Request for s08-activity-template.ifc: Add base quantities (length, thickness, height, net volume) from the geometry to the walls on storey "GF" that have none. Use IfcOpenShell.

First a look at what the model holds.

```python
import ifcopenshell
import ifcopenshell.util.element
import ifcopenshell.util.unit

model = ifcopenshell.open("s08-activity-template.ifc")
print(model.schema)
for unit_type in ("LENGTHUNIT", "AREAUNIT", "VOLUMEUNIT"):
    print(unit_type, ifcopenshell.util.unit.calculate_unit_scale(model, unit_type))
storey = next(s for s in model.by_type("IfcBuildingStorey") if s.Name == "GF")
walls = [e for e in ifcopenshell.util.element.get_decomposition(storey) if e.is_a("IfcWall")]
for e in sorted(walls, key=lambda e: e.id()):
    print(e.id(), e.is_a(), e.Name, list(ifcopenshell.util.element.get_psets(e, qtos_only=True)), sep=" | ")
```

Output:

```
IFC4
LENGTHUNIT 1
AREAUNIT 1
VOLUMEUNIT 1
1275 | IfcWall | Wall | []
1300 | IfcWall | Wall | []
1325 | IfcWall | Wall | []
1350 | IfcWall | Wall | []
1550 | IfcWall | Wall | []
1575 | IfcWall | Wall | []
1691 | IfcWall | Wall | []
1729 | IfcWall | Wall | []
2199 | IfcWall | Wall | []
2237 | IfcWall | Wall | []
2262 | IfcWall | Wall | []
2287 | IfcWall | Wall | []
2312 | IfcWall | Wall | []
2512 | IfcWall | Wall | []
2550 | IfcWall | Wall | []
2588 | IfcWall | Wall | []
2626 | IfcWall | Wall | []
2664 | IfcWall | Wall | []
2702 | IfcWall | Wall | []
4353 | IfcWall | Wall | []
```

```python
import ifcopenshell
import ifcopenshell.api.pset
import ifcopenshell.geom
import ifcopenshell.util.element
import ifcopenshell.util.shape
import ifcopenshell.util.unit

model = ifcopenshell.open("s08-activity-template.ifc")
unit_scale = ifcopenshell.util.unit.calculate_unit_scale(model)
volume_scale = ifcopenshell.util.unit.calculate_unit_scale(model, "VOLUMEUNIT")
settings = ifcopenshell.geom.settings()

storey = next(s for s in model.by_type("IfcBuildingStorey") if s.Name == "GF")
walls = [e for e in ifcopenshell.util.element.get_decomposition(storey) if e.is_a("IfcWall")]

for e in sorted(walls, key=lambda e: e.id()):
    if ifcopenshell.util.element.get_psets(e, qtos_only=True, should_inherit=False):
        continue
    # Geometry comes back in metres, in the element's own axes.
    shape = ifcopenshell.geom.create_shape(settings, e)
    values = {
        "Length": ifcopenshell.util.shape.get_x(shape.geometry) / unit_scale,
        "Width": ifcopenshell.util.shape.get_y(shape.geometry) / unit_scale,
        "Height": ifcopenshell.util.shape.get_z(shape.geometry) / unit_scale,
        "NetVolume": ifcopenshell.util.shape.get_volume(shape.geometry) / volume_scale,
    }
    qto = ifcopenshell.api.pset.add_qto(model, product=e, name="Qto_WallBaseQuantities")
    ifcopenshell.api.pset.edit_qto(model, qto=qto, properties=values)
    print(e.id(), {k: round(v, 3) for k, v in values.items()})

model.write("s08-activity-template_rev.ifc")
```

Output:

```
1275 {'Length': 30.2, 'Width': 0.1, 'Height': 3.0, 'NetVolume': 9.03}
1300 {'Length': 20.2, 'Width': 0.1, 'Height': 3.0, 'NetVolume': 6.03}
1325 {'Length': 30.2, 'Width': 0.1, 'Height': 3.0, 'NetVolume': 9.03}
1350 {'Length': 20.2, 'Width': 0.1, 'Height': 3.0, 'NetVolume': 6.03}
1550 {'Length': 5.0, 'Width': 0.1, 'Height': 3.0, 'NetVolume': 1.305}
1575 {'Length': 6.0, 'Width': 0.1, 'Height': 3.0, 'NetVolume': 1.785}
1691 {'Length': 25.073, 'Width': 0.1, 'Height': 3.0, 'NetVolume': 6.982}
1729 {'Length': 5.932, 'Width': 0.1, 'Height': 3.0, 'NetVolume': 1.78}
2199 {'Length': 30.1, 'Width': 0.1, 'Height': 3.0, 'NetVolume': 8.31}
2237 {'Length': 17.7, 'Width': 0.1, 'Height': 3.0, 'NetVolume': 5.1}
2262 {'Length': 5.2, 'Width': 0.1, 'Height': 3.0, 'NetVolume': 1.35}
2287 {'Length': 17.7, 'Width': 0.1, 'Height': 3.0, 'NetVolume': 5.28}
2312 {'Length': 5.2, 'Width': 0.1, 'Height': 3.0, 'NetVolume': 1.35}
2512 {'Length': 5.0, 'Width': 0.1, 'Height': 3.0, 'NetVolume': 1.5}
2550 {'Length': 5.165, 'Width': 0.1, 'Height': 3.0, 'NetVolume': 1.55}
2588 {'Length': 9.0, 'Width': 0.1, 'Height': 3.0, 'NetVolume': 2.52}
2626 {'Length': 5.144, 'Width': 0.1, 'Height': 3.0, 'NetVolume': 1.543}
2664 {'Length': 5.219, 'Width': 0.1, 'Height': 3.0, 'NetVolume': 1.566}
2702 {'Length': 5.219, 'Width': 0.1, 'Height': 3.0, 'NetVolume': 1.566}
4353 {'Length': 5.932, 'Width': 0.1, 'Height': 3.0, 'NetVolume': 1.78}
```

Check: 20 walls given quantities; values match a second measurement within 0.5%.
